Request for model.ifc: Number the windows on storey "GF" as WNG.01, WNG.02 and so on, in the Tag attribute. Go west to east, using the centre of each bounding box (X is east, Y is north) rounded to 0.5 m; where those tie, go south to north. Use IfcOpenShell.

First a look at what the model holds.

```python
import ifcopenshell
import ifcopenshell.util.element
import ifcopenshell.util.placement

model = ifcopenshell.open("model.ifc")
print(model.schema)
storey = next(s for s in model.by_type("IfcBuildingStorey") if s.Name == "GF")
windows = [e for e in ifcopenshell.util.element.get_decomposition(storey) if e.is_a("IfcWindow")]
for e in sorted(windows, key=lambda e: e.id()):
    origin = ifcopenshell.util.placement.get_local_placement(e.ObjectPlacement)[:3, 3]
    print(e.id(), e.Tag, e.Name, origin.round(2) + 0.0, sep=" | ")
```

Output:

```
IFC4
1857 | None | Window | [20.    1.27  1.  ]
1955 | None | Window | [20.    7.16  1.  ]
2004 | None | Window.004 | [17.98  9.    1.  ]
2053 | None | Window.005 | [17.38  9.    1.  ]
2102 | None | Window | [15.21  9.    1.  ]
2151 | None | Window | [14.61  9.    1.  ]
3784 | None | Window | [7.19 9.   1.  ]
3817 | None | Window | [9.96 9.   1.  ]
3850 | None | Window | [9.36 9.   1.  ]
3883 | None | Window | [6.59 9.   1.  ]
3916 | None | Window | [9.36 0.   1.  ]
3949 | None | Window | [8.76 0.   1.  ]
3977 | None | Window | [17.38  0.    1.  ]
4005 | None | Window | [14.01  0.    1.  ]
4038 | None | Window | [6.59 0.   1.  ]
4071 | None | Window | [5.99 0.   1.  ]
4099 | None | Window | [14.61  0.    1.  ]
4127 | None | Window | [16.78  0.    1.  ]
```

```python
import ifcopenshell
import ifcopenshell.geom
import ifcopenshell.util.element
import ifcopenshell.util.shape

model = ifcopenshell.open("model.ifc")
settings = ifcopenshell.geom.settings()
settings.set("use-world-coords", True)


def centre(element):
    shape = ifcopenshell.geom.create_shape(settings, element)
    return ifcopenshell.util.shape.get_bbox_centroid(shape.geometry)


storey = next(s for s in model.by_type("IfcBuildingStorey") if s.Name == "GF")
windows = [e for e in ifcopenshell.util.element.get_decomposition(storey) if e.is_a("IfcWindow")]

# Insertion points can sit at a corner or the storey origin, so sort by the geometry (in metres).
centres = {e: centre(e) for e in windows}
windows.sort(key=lambda e: (round(centres[e][0] / 0.5), centres[e][1]))

for i, e in enumerate(windows, start=1):
    number = f"WNG.{i:02d}"
    e.Tag = number
    print(e.id(), number)

model.write("model-out.ifc")
```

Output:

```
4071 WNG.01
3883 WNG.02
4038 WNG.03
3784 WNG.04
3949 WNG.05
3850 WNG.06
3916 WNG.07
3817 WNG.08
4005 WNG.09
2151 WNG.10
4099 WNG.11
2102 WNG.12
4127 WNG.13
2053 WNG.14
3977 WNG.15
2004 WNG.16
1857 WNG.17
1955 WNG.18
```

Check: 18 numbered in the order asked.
